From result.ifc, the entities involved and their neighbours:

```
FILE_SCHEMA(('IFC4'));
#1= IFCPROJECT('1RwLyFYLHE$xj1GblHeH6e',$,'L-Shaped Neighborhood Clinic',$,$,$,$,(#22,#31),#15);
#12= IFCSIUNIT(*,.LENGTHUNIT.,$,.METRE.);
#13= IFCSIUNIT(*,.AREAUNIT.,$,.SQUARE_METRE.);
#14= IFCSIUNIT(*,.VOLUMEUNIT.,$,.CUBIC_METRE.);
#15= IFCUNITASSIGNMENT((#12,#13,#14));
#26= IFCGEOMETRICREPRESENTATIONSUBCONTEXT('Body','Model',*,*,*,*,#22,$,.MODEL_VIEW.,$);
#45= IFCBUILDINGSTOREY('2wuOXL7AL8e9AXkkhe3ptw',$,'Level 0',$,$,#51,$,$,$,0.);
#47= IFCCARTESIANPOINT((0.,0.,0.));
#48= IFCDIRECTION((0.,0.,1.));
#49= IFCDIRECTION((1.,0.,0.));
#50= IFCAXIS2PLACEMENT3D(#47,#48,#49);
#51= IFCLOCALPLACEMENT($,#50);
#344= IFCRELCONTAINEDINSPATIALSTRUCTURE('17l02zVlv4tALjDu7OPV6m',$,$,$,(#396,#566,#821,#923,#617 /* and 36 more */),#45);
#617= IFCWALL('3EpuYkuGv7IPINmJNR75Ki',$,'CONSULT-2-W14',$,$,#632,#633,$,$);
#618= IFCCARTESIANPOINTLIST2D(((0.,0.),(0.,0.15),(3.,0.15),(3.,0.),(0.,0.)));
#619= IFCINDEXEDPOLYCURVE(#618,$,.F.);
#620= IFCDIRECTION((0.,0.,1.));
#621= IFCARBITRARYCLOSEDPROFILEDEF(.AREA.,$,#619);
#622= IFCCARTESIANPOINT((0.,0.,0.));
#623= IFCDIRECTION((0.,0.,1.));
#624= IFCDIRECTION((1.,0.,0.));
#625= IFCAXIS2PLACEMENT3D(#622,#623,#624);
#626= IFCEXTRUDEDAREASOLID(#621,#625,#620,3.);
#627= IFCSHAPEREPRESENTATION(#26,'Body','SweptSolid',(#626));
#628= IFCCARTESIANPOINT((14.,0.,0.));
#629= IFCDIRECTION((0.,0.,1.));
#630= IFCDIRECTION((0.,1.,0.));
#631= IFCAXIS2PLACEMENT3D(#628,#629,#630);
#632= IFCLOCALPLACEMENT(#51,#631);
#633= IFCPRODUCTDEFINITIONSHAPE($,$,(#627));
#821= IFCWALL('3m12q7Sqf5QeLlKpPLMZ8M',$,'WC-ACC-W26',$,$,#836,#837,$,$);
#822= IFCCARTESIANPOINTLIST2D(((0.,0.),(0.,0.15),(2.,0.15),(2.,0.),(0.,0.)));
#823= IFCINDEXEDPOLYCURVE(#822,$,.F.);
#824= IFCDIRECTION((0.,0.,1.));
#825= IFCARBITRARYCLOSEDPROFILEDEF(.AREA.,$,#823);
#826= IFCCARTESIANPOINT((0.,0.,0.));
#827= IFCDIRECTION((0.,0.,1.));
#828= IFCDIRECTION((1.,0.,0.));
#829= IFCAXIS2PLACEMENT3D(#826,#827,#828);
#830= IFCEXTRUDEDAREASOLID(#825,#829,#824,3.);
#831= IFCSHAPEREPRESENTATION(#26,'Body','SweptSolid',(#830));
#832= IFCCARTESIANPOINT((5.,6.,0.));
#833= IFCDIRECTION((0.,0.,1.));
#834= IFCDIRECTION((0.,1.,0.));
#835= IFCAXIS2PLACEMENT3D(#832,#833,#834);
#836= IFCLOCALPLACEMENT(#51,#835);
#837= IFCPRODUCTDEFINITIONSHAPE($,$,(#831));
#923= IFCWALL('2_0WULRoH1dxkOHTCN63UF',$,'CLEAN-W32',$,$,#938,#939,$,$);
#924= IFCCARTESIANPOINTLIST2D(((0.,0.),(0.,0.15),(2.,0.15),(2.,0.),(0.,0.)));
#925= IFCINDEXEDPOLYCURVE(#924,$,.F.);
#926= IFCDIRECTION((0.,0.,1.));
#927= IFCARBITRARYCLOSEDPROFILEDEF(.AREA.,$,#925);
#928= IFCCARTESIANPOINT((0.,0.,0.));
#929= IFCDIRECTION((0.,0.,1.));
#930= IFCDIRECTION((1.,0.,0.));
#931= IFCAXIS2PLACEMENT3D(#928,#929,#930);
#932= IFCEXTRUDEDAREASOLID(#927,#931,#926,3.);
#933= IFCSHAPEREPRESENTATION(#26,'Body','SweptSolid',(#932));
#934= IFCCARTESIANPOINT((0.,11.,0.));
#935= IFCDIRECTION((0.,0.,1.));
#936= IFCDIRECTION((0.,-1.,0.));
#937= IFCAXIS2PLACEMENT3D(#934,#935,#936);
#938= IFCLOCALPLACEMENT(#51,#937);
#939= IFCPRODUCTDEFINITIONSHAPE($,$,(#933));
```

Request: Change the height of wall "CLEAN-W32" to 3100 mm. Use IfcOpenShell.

```python
import ifcopenshell
import ifcopenshell.geom
import ifcopenshell.util.representation
import ifcopenshell.util.shape
import ifcopenshell.util.unit

model = ifcopenshell.open("result.ifc")
unit_scale = ifcopenshell.util.unit.calculate_unit_scale(model)
settings = ifcopenshell.geom.settings()


def volume(element):
    """Net volume in cubic metres, openings subtracted."""
    shape = ifcopenshell.geom.create_shape(settings, element)
    return ifcopenshell.util.shape.get_volume(shape.geometry)


wall = model.by_guid("2_0WULRoH1dxkOHTCN63UF")
before = volume(wall)

body = ifcopenshell.util.representation.get_representation(wall, "Model", "Body")
solid = body.Items[0]
old_height = solid.Depth
solid.Depth = 3.1 / unit_scale
after = volume(wall)

print(f"height {old_height:g} -> {solid.Depth:g}, volume {before:.3f} -> {after:.3f} m3")

model.write("result_edited.ifc")
```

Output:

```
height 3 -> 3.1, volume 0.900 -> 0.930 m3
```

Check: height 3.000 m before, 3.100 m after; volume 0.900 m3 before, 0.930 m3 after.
